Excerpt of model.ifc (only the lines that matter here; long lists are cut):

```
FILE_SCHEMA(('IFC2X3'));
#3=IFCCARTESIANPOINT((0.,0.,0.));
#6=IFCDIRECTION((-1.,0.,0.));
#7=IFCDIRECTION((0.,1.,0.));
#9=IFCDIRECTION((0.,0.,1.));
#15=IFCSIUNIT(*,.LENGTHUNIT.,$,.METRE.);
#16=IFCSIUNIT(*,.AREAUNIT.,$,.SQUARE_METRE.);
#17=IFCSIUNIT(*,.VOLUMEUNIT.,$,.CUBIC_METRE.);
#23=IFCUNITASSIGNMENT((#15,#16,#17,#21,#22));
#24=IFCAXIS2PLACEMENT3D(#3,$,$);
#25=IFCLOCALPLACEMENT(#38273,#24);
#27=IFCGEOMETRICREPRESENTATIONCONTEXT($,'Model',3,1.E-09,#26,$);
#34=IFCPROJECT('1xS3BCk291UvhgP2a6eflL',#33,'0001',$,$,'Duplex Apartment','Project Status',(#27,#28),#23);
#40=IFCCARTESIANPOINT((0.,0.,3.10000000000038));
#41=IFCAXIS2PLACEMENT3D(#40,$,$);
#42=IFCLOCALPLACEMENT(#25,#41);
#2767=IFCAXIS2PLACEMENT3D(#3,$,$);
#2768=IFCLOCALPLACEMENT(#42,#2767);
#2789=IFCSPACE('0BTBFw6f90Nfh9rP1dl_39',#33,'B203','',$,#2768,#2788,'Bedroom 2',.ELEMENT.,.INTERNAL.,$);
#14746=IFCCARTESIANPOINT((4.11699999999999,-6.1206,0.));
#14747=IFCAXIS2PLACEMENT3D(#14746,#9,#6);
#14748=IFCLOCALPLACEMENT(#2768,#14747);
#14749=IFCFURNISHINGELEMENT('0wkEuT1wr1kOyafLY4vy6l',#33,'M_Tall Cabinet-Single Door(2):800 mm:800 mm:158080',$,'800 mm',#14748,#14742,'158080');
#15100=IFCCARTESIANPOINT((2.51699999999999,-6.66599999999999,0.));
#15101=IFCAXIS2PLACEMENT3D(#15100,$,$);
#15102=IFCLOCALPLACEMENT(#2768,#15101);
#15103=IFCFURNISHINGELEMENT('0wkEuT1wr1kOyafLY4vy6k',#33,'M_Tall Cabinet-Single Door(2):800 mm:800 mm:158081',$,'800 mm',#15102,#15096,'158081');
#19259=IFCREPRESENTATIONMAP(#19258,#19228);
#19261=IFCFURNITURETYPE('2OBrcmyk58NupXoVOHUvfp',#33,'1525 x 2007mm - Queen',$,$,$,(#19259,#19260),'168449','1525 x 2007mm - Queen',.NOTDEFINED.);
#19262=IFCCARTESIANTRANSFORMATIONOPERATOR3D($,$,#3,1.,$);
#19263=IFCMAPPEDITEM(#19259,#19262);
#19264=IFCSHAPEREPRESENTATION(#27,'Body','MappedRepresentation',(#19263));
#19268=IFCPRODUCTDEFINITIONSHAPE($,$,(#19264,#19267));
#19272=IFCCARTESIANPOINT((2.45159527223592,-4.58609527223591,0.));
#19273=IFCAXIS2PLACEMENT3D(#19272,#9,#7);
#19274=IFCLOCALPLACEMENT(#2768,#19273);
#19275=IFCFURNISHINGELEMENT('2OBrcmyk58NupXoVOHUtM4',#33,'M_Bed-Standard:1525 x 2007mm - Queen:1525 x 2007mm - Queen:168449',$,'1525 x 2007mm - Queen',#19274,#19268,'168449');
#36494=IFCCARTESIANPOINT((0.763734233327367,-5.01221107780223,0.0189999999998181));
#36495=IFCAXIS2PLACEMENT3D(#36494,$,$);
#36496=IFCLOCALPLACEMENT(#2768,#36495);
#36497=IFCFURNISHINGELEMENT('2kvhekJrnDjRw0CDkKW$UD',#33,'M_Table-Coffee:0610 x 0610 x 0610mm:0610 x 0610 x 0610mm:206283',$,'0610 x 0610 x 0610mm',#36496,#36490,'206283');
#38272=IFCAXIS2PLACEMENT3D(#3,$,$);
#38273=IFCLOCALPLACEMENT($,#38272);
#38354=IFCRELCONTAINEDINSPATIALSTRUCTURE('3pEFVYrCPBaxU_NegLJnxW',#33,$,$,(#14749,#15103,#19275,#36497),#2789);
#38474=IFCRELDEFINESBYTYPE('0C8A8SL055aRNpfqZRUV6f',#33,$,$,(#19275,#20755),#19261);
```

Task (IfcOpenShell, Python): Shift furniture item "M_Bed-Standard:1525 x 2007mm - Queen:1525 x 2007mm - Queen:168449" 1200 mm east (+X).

```python
import ifcopenshell
import ifcopenshell.api.geometry
import ifcopenshell.util.placement

model = ifcopenshell.open("model.ifc")

item = model.by_guid("2OBrcmyk58NupXoVOHUtM4")
matrix = ifcopenshell.util.placement.get_local_placement(item.ObjectPlacement)
matrix[0, 3] += 1.2
ifcopenshell.api.geometry.edit_object_placement(model, product=item, matrix=matrix, is_si=False)

print(ifcopenshell.util.placement.get_local_placement(item.ObjectPlacement).round(3) + 0.0)

model.write("model-out.ifc")
```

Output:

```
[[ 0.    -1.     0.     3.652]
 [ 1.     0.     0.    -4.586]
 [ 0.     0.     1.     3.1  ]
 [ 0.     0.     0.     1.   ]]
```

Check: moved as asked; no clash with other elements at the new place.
